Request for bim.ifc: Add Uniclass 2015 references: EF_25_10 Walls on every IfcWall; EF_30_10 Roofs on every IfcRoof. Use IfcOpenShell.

First a look at what the model holds.

```python
import ifcopenshell

model = ifcopenshell.open("bim.ifc")
print(model.schema)
print("classifications:", [c.Name for c in model.by_type("IfcClassification")])
for ifc_class in ("IfcDoor", "IfcRoof", "IfcStair", "IfcWall", "IfcWindow"):
    print(ifc_class, len(model.by_type(ifc_class)))
```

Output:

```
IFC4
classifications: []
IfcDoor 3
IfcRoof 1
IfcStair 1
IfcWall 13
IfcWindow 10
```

```python
import ifcopenshell
import ifcopenshell.api.classification

model = ifcopenshell.open("bim.ifc")

system = ifcopenshell.api.classification.add_classification(model, classification="Uniclass 2015")

codes = {
    "IfcWall": ("EF_25_10", "Walls"),
    "IfcRoof": ("EF_30_10", "Roofs"),
}
for ifc_class, (code, name) in codes.items():
    products = model.by_type(ifc_class)
    ifcopenshell.api.classification.add_reference(
        model, products=products, classification=system, identification=code, name=name
    )
    print(code, len(products))

model.write("bim-out.ifc")
```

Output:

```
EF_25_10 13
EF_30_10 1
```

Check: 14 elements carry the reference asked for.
